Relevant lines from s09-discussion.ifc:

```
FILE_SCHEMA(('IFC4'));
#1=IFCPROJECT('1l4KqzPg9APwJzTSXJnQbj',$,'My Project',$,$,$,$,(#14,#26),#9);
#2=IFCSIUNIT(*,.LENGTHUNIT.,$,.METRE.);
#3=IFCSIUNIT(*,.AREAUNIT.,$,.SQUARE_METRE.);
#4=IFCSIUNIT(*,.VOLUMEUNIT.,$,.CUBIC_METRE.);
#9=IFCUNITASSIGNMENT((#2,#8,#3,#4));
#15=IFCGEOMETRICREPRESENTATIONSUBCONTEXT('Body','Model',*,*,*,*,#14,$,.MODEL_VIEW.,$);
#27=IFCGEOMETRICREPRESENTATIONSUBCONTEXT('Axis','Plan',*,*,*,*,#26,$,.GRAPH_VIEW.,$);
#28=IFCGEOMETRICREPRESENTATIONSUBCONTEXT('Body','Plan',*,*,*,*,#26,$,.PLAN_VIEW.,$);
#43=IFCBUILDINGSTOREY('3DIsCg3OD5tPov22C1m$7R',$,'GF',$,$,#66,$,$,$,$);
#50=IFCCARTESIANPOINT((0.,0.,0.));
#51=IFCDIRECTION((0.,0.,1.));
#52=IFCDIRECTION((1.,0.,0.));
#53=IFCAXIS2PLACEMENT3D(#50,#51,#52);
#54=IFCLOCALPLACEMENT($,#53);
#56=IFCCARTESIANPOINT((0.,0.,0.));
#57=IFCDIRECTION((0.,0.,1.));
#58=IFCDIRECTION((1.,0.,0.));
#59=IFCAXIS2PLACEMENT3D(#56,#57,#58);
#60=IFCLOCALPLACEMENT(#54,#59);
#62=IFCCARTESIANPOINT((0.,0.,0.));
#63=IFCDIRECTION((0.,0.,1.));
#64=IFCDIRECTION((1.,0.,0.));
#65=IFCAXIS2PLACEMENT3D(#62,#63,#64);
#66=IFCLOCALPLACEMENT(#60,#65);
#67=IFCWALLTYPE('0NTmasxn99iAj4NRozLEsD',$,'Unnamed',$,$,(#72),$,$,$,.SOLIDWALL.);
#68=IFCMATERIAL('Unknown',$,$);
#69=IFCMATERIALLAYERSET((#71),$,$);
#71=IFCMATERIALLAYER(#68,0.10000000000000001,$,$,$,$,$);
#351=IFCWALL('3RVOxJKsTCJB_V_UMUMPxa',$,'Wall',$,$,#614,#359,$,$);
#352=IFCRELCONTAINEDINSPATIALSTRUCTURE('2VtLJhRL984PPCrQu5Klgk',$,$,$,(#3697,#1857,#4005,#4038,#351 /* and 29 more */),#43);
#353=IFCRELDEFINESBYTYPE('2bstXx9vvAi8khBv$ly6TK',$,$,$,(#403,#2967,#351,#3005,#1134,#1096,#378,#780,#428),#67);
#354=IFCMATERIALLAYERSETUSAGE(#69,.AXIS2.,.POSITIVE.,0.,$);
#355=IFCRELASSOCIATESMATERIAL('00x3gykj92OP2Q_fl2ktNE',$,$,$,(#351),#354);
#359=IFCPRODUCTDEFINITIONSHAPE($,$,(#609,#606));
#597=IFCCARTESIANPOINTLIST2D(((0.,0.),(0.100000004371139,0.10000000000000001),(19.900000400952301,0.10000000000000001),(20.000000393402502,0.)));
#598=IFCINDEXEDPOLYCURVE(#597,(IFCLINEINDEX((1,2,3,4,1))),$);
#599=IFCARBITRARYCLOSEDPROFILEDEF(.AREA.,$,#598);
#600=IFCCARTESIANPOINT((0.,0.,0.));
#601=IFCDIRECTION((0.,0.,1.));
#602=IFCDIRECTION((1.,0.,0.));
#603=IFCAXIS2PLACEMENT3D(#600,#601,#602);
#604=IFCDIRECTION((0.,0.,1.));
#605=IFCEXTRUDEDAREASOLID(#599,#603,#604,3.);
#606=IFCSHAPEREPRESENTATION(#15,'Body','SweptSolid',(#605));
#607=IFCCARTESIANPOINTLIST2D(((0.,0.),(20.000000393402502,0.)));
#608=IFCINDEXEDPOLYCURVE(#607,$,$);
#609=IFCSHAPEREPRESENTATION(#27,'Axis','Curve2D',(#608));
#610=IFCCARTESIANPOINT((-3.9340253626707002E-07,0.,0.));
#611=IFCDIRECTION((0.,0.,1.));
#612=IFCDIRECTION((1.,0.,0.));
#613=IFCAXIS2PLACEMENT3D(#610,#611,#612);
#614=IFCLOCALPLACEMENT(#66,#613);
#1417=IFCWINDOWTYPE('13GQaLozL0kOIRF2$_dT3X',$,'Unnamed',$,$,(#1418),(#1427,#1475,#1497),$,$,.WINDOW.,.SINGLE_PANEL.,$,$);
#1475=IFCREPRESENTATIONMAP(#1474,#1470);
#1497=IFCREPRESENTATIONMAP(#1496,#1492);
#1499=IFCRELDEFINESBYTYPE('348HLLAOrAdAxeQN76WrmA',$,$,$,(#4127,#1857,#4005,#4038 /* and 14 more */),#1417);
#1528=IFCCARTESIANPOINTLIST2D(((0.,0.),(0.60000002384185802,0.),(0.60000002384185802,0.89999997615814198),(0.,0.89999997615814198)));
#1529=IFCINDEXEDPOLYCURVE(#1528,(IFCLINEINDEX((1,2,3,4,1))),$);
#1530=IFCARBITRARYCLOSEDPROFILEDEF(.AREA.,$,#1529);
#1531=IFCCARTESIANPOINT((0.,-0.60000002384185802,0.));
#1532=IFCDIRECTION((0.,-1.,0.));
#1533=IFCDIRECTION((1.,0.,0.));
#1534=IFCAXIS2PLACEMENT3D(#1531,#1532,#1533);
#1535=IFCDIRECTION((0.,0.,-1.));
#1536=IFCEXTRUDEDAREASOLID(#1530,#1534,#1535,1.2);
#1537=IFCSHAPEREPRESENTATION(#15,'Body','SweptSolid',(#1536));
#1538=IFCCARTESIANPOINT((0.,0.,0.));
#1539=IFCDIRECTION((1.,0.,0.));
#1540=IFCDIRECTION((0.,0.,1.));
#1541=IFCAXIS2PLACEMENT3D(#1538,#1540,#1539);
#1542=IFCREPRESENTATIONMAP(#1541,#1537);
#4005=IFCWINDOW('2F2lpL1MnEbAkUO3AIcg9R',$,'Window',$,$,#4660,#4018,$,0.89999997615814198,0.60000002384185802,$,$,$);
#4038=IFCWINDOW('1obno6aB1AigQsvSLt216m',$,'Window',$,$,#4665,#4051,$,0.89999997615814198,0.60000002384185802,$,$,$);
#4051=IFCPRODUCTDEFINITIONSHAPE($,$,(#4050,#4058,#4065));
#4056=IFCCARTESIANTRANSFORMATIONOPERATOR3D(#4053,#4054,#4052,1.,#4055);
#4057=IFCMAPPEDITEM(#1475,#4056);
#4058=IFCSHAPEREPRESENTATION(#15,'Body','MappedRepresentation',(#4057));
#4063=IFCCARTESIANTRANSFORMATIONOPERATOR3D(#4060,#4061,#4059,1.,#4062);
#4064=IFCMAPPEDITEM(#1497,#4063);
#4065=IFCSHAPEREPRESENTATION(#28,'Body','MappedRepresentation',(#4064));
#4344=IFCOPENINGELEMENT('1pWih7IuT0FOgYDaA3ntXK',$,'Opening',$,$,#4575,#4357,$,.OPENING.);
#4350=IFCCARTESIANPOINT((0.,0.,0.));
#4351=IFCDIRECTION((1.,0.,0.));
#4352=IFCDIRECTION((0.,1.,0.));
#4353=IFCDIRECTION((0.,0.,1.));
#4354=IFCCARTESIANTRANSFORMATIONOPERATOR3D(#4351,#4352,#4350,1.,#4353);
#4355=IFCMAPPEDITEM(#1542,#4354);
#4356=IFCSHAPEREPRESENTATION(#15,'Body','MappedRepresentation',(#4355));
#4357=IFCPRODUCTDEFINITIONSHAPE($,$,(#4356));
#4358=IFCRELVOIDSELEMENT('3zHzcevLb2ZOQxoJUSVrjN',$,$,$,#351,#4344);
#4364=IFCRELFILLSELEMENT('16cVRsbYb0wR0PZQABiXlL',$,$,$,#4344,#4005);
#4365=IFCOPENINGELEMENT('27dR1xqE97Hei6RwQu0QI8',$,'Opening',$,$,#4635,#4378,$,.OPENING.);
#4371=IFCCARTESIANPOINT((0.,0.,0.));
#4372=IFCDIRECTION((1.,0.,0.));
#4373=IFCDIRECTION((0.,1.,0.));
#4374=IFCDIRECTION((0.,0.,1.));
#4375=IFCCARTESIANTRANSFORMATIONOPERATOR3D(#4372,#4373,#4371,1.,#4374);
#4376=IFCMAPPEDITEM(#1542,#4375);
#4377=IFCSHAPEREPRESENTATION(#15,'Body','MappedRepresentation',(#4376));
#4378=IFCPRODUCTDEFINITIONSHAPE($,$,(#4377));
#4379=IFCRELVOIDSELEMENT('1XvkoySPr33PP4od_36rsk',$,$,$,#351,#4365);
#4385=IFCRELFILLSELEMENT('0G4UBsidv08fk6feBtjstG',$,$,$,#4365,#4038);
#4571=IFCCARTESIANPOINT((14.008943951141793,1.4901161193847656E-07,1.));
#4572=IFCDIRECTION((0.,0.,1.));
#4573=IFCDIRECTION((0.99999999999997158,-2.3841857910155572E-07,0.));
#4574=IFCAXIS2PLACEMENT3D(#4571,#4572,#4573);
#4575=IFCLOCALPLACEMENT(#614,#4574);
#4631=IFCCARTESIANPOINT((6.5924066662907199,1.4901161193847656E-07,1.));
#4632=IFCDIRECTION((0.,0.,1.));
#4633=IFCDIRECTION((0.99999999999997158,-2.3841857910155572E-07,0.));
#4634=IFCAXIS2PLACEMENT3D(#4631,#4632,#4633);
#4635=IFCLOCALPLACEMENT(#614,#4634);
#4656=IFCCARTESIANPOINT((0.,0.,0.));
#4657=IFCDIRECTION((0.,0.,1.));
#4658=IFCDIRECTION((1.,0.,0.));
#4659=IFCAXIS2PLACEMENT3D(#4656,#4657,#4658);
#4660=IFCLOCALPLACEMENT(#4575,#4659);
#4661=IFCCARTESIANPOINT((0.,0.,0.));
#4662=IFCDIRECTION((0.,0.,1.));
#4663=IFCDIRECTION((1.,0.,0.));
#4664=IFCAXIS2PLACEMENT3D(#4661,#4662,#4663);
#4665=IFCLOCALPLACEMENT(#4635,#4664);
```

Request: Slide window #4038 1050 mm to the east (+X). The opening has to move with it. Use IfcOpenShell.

```python
import ifcopenshell
import ifcopenshell.api.geometry
import ifcopenshell.util.placement
import ifcopenshell.util.unit

model = ifcopenshell.open("s09-discussion.ifc")
unit_scale = ifcopenshell.util.unit.calculate_unit_scale(model)

window = model.by_id(4038)
opening = window.FillsVoids[0].RelatingOpeningElement
wall = opening.VoidsElements[0].RelatingBuildingElement

wall_matrix = ifcopenshell.util.placement.get_local_placement(wall.ObjectPlacement)
shift = wall_matrix[:3, 0] * 1.05 / unit_scale
before = ifcopenshell.util.placement.get_local_placement(window.ObjectPlacement)[:3, 3].copy()

# The window is placed relative to its opening, so it follows when the opening moves.
matrix = ifcopenshell.util.placement.get_local_placement(opening.ObjectPlacement)
matrix[:3, 3] += shift
ifcopenshell.api.geometry.edit_object_placement(
    model, product=opening, matrix=matrix, is_si=False, should_transform_children=True
)

after = ifcopenshell.util.placement.get_local_placement(window.ObjectPlacement)[:3, 3]
print("window moved by", (after - before).round(3) + 0.0)

model.write("s09-discussion-out.ifc")
```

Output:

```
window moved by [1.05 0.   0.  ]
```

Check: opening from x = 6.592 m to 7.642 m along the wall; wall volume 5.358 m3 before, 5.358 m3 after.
